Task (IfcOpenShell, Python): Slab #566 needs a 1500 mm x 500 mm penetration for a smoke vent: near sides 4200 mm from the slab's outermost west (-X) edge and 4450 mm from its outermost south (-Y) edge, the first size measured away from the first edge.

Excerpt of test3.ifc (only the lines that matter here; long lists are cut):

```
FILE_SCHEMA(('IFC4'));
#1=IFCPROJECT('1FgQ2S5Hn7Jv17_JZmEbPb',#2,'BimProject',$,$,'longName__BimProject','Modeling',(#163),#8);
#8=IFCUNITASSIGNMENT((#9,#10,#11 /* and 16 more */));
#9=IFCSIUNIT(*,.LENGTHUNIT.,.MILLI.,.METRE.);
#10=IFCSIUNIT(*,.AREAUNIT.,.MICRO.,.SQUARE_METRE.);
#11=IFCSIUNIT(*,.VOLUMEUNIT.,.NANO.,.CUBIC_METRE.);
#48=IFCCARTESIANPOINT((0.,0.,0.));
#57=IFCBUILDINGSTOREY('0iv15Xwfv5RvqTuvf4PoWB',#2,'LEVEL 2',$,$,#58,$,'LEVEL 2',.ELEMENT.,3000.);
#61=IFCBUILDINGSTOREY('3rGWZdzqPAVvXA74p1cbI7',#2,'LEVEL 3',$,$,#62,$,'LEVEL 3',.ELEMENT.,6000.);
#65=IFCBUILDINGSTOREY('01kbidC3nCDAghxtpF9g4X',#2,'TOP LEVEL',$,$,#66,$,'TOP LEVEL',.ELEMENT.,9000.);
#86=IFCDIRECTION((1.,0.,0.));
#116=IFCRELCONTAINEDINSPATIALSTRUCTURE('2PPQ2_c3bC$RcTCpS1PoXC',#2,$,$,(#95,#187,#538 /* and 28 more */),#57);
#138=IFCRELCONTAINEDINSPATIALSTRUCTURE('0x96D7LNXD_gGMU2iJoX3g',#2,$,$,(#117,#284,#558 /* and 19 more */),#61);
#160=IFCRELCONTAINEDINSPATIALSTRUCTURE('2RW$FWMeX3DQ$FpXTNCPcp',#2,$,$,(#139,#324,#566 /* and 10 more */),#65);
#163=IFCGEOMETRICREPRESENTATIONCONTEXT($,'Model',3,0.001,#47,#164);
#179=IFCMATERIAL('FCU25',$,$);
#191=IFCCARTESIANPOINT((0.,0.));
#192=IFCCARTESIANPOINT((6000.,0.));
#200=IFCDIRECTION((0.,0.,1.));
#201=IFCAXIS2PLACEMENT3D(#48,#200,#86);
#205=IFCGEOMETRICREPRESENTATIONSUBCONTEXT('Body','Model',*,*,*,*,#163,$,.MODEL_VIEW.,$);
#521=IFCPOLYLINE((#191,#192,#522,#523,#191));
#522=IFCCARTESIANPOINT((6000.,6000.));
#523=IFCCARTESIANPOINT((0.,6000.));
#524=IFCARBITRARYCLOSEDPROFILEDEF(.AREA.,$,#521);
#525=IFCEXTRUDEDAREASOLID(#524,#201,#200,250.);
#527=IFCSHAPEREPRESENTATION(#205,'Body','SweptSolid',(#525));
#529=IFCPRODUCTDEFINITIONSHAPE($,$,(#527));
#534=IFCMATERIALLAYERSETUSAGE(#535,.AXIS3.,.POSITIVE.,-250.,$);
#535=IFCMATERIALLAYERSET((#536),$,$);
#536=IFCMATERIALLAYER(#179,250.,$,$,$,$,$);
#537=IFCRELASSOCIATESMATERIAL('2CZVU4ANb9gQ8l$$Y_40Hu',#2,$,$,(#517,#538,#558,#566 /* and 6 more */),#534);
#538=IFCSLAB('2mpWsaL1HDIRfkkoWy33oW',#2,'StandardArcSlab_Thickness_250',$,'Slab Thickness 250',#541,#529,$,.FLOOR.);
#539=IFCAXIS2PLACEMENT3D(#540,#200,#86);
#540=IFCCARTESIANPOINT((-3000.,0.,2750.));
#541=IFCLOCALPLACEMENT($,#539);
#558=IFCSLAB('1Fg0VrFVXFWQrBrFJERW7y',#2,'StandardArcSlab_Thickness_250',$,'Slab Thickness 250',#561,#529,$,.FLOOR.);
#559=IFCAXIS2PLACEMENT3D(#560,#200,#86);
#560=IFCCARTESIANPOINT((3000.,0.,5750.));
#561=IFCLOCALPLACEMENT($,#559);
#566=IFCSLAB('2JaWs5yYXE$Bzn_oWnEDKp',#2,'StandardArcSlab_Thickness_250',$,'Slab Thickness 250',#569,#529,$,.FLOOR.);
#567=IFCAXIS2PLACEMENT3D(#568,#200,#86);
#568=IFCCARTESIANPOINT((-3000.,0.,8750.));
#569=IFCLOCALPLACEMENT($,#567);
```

```python
import numpy as np
import ifcopenshell
import ifcopenshell.api.feature
import ifcopenshell.api.geometry
import ifcopenshell.api.root
import ifcopenshell.geom
import ifcopenshell.util.placement
import ifcopenshell.util.representation
import ifcopenshell.util.shape
import ifcopenshell.util.unit

model = ifcopenshell.open("test3.ifc")
unit_scale = ifcopenshell.util.unit.calculate_unit_scale(model)
settings = ifcopenshell.geom.settings()


def volume(element):
    """Net volume in cubic metres, openings subtracted."""
    shape = ifcopenshell.geom.create_shape(settings, element)
    return ifcopenshell.util.shape.get_volume(shape.geometry)


slab = model.by_guid("2JaWs5yYXE$Bzn_oWnEDKp")
before = volume(slab)

# Extent in the slab's own axes, in metres. The edges named are its -X and -Y sides.
slab_shape = ifcopenshell.geom.create_shape(settings, slab)
vertices = ifcopenshell.util.shape.get_vertices(slab_shape.geometry)
x_min, y_min, bottom = vertices.min(axis=0)
top = vertices[:, 2].max()

opening = ifcopenshell.api.root.create_entity(model, ifc_class="IfcOpeningElement", name="Smoke vent opening", predefined_type="OPENING")
context = ifcopenshell.util.representation.get_context(model, "Model", "Body", "MODEL_VIEW")
width, depth = 1.5, 0.5
outline = [(0.0, 0.0), (width, 0.0), (width, depth), (0.0, depth), (0.0, 0.0)]
# Overshoot both faces by 50 mm so the cut is clean.
shape = ifcopenshell.api.geometry.add_slab_representation(
    model, context=context, depth=top - bottom + 0.1, polyline=outline
)
ifcopenshell.api.geometry.assign_representation(model, product=opening, representation=shape)

matrix = ifcopenshell.util.placement.get_local_placement(slab.ObjectPlacement)
matrix[:, 3] = matrix @ np.append(np.array([x_min + 4.2, y_min + 4.45, bottom - 0.05]) / unit_scale, 1.0)
ifcopenshell.api.geometry.edit_object_placement(model, product=opening, matrix=matrix, is_si=False)
ifcopenshell.api.feature.add_feature(model, feature=opening, element=slab)

after = volume(slab)

print(f"slab volume {before:.3f} -> {after:.3f} m3")

model.write("test3_edited.ifc")
```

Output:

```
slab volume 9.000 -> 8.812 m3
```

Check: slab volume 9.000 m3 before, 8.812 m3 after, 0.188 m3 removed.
